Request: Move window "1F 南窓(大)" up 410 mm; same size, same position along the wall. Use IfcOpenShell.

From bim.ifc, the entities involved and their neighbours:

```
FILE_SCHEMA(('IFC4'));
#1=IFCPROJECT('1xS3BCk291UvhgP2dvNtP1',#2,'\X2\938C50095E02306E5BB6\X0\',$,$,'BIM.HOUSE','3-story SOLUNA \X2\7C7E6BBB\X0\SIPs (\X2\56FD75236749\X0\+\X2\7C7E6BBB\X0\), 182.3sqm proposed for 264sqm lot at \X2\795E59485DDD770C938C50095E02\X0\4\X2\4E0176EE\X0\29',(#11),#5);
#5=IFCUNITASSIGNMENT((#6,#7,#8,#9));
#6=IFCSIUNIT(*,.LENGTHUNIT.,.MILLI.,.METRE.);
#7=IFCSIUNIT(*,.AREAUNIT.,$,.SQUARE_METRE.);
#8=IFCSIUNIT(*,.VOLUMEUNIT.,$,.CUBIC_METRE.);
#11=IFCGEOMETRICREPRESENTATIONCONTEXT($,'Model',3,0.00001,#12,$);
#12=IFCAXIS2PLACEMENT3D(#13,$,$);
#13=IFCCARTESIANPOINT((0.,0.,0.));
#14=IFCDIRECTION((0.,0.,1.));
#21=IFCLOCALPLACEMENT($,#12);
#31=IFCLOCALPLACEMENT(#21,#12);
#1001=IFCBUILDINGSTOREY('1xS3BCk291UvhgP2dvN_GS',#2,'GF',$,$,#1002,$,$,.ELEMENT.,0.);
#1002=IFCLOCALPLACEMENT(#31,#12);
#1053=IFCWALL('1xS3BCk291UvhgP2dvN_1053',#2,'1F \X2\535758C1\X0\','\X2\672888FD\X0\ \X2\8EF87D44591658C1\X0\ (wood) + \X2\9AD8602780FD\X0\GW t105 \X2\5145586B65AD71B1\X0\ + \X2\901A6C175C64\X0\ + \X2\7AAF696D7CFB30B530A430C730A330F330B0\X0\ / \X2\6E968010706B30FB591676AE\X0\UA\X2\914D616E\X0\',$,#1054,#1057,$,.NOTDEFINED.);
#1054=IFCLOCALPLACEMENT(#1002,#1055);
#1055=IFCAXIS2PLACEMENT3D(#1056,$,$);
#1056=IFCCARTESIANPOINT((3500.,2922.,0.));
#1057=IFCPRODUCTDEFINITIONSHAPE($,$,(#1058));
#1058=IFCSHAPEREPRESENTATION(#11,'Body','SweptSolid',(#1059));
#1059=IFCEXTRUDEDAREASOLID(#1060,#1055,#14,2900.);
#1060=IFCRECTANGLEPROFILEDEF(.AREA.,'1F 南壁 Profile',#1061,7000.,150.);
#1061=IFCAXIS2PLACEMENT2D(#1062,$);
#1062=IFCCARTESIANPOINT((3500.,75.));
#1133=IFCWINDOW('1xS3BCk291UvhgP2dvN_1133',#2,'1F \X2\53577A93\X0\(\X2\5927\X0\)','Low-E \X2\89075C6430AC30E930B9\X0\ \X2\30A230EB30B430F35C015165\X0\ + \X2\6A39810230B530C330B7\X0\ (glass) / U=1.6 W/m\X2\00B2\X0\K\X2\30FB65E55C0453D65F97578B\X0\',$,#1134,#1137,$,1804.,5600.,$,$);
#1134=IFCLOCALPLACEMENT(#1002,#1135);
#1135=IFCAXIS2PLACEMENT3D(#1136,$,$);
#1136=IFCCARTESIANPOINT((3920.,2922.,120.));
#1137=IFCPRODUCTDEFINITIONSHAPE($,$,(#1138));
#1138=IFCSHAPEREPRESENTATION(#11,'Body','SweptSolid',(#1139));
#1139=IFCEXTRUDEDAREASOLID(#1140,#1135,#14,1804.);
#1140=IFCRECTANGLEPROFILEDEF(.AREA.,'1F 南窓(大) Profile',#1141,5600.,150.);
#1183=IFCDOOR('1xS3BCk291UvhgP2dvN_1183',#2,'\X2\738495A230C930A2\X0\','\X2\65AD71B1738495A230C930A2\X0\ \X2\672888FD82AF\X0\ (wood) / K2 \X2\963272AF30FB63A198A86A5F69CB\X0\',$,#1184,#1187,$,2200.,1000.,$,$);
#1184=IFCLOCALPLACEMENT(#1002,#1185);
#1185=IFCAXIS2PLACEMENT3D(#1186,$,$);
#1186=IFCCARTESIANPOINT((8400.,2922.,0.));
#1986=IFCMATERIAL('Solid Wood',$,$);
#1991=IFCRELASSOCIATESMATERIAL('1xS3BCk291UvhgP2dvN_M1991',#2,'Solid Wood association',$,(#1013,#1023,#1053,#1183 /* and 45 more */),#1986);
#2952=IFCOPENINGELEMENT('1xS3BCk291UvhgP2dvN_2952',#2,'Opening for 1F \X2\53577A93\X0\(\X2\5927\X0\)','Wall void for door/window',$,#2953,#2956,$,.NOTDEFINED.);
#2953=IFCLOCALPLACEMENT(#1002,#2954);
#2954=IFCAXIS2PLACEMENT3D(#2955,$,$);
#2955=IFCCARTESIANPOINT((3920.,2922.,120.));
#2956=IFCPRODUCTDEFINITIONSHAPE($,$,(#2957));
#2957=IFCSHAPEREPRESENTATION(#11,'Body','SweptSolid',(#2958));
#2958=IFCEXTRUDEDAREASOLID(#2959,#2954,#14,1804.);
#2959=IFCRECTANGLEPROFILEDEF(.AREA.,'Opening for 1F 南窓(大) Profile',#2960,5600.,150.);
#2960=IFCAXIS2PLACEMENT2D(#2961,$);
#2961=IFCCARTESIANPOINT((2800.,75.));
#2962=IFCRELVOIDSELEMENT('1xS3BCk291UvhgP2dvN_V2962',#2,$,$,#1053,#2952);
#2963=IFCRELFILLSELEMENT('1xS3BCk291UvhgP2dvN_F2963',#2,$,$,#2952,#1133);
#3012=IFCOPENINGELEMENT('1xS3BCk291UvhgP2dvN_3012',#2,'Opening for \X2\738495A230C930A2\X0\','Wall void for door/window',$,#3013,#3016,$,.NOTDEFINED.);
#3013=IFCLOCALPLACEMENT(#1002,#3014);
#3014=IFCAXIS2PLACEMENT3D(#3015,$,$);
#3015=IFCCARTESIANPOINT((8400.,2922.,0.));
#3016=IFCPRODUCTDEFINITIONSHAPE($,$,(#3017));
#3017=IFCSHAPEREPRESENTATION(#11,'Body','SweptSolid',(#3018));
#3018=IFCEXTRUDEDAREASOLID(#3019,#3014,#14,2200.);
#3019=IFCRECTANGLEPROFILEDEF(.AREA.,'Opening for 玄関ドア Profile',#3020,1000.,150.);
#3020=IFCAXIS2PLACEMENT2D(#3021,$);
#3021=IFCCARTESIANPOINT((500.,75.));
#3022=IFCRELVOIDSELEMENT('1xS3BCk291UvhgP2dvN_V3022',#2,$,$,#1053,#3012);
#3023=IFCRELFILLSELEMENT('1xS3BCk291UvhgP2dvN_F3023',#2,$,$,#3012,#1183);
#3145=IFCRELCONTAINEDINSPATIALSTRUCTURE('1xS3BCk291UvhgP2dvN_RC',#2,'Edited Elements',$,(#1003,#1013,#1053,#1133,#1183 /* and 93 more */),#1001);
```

```python
import numpy as np
import ifcopenshell
import ifcopenshell.api.geometry
import ifcopenshell.util.placement
import ifcopenshell.util.unit

model = ifcopenshell.open("bim.ifc")
unit_scale = ifcopenshell.util.unit.calculate_unit_scale(model)

window = model.by_guid("1xS3BCk291UvhgP2dvN_1133")
opening = window.FillsVoids[0].RelatingOpeningElement
dz = 0.41 / unit_scale

shift = np.array([0.0, 0.0, dz])
# The window is not placed relative to its opening, so move both.
for product in (opening, window):
    matrix = ifcopenshell.util.placement.get_local_placement(product.ObjectPlacement)
    matrix[:3, 3] += shift
    ifcopenshell.api.geometry.edit_object_placement(model, product=product, matrix=matrix, is_si=False)

print(f"moved by {dz * unit_scale:+.3f} m")

model.write("bim-out.ifc")
```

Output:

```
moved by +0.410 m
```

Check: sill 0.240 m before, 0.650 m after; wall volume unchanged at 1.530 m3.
